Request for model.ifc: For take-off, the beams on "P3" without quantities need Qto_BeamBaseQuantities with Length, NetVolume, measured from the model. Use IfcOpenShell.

First a look at what the model holds.

```python
import ifcopenshell
import ifcopenshell.util.element
import ifcopenshell.util.unit

model = ifcopenshell.open("model.ifc")
print(model.schema)
for unit_type in ("LENGTHUNIT", "AREAUNIT", "VOLUMEUNIT"):
    print(unit_type, ifcopenshell.util.unit.calculate_unit_scale(model, unit_type))
storey = next(s for s in model.by_type("IfcBuildingStorey") if s.Name == "P3")
beams = [e for e in ifcopenshell.util.element.get_decomposition(storey) if e.is_a("IfcBeam")]
for e in sorted(beams, key=lambda e: e.id()):
    print(e.id(), e.is_a(), e.Name, list(ifcopenshell.util.element.get_psets(e, qtos_only=True)), sep=" | ")
```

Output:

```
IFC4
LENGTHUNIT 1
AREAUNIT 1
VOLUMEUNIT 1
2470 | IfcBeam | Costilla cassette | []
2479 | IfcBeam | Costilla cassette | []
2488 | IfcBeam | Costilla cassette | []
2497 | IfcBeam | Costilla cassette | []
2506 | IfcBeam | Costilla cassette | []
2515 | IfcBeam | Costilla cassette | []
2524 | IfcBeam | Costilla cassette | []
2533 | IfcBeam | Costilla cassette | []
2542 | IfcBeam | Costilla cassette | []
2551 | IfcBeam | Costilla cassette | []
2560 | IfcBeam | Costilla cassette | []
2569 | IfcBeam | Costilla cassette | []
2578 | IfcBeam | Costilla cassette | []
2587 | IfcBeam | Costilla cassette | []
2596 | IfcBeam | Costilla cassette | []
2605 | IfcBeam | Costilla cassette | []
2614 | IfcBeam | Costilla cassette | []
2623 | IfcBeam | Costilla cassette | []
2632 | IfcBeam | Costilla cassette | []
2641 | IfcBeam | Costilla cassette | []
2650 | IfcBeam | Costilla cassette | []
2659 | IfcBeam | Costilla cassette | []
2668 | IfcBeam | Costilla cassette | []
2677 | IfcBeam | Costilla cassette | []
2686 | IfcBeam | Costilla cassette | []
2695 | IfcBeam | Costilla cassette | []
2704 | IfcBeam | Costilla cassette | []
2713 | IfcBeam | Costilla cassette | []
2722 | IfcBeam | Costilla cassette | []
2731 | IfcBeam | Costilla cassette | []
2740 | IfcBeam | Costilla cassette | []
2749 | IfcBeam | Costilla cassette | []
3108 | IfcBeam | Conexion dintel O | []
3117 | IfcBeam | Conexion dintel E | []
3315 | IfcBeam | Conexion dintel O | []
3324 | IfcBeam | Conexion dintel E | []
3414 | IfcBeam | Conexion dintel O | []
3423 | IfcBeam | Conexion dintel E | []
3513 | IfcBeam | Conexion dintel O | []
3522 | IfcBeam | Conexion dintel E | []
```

```python
import ifcopenshell
import ifcopenshell.api.pset
import ifcopenshell.geom
import ifcopenshell.util.element
import ifcopenshell.util.shape
import ifcopenshell.util.unit

model = ifcopenshell.open("model.ifc")
unit_scale = ifcopenshell.util.unit.calculate_unit_scale(model)
volume_scale = ifcopenshell.util.unit.calculate_unit_scale(model, "VOLUMEUNIT")
settings = ifcopenshell.geom.settings()

storey = next(s for s in model.by_type("IfcBuildingStorey") if s.Name == "P3")
beams = [e for e in ifcopenshell.util.element.get_decomposition(storey) if e.is_a("IfcBeam")]

for e in sorted(beams, key=lambda e: e.id()):
    if ifcopenshell.util.element.get_psets(e, qtos_only=True, should_inherit=False):
        continue
    # Geometry comes back in metres, in the element's own axes.
    shape = ifcopenshell.geom.create_shape(settings, e)
    values = {
        "Length": ifcopenshell.util.shape.get_max_xyz(shape.geometry) / unit_scale,
        "NetVolume": ifcopenshell.util.shape.get_volume(shape.geometry) / volume_scale,
    }
    qto = ifcopenshell.api.pset.add_qto(model, product=e, name="Qto_BeamBaseQuantities")
    ifcopenshell.api.pset.edit_qto(model, qto=qto, properties=values)
    print(e.id(), {k: round(v, 3) for k, v in values.items()})

model.write("model_edited.ifc")
```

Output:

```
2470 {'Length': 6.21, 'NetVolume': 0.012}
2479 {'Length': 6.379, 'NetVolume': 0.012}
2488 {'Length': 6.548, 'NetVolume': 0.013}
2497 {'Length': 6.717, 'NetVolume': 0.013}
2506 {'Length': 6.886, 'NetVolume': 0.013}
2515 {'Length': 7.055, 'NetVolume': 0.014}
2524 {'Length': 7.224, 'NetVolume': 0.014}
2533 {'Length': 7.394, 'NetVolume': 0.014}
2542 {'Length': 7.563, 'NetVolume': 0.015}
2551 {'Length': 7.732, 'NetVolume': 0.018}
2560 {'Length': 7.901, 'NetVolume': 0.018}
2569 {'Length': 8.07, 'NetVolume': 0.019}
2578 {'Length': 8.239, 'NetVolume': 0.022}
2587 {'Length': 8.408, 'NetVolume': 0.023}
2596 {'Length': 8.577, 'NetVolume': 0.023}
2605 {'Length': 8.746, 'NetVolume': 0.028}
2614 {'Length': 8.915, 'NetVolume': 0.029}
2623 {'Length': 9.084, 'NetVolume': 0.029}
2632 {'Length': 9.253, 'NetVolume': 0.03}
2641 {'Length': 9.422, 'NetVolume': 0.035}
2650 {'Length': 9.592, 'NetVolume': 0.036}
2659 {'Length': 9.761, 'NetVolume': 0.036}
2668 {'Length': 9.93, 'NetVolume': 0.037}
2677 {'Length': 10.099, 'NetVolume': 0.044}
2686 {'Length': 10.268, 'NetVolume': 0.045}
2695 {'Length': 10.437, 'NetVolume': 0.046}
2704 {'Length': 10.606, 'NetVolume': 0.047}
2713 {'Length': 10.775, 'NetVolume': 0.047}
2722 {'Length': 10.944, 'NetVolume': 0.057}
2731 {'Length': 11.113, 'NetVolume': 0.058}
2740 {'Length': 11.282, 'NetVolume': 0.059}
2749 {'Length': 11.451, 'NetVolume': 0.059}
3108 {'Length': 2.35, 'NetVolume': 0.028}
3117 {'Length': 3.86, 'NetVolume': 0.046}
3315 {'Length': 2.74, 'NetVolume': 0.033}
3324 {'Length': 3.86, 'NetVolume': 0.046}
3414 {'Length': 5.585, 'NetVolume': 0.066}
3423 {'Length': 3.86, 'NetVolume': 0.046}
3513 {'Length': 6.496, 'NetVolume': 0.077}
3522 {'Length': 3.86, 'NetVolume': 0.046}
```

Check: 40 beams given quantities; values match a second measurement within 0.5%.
